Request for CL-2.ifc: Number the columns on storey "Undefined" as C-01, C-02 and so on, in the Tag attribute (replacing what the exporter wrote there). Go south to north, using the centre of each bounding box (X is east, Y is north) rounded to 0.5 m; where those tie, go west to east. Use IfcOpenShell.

First a look at what the model holds.

```python
import ifcopenshell
import ifcopenshell.util.element
import ifcopenshell.util.placement

model = ifcopenshell.open("CL-2.ifc")
print(model.schema)
storey = next(s for s in model.by_type("IfcBuildingStorey") if s.Name == "Undefined")
columns = [e for e in ifcopenshell.util.element.get_decomposition(storey) if e.is_a("IfcColumn")]
for e in sorted(columns, key=lambda e: e.id()):
    origin = ifcopenshell.util.placement.get_local_placement(e.ObjectPlacement)[:3, 3]
    print(e.id(), e.Tag, e.Name, origin.round(2) + 0.0, sep=" | ")
```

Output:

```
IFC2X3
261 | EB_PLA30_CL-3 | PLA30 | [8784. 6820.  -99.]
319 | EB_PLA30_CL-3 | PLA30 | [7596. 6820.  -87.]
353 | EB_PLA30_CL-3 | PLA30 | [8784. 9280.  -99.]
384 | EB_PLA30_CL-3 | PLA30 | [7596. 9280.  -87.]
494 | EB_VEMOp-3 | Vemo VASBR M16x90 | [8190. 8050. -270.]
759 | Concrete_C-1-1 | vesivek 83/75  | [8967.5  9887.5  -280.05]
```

```python
import ifcopenshell
import ifcopenshell.geom
import ifcopenshell.util.element
import ifcopenshell.util.shape

model = ifcopenshell.open("CL-2.ifc")
settings = ifcopenshell.geom.settings()
settings.set("use-world-coords", True)


def centre(element):
    shape = ifcopenshell.geom.create_shape(settings, element)
    return ifcopenshell.util.shape.get_bbox_centroid(shape.geometry)


storey = next(s for s in model.by_type("IfcBuildingStorey") if s.Name == "Undefined")
columns = [e for e in ifcopenshell.util.element.get_decomposition(storey) if e.is_a("IfcColumn")]

# Insertion points can sit at a corner or the storey origin, so sort by the geometry (in metres).
centres = {e: centre(e) for e in columns}
columns.sort(key=lambda e: (round(centres[e][1] / 0.5), centres[e][0]))

for i, e in enumerate(columns, start=1):
    number = f"C-{i:02d}"
    e.Tag = number
    print(e.id(), number)

model.write("CL-2_v2.ifc")
```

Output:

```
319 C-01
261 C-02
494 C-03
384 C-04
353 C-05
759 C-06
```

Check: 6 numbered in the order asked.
